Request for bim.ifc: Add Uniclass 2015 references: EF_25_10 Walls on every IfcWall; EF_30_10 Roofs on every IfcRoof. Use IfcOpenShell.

First a look at what the model holds.

```python
import ifcopenshell

model = ifcopenshell.open("bim.ifc")
print(model.schema)
print("classifications:", [c.Name for c in model.by_type("IfcClassification")])
for ifc_class in ("IfcDoor", "IfcRoof", "IfcStair", "IfcWall", "IfcWindow"):
    print(ifc_class, len(model.by_type(ifc_class)))
```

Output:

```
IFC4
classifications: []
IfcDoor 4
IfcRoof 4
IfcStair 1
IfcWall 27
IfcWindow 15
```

```python
import ifcopenshell
import ifcopenshell.api.classification

model = ifcopenshell.open("bim.ifc")

system = ifcopenshell.api.classification.add_classification(model, classification="Uniclass 2015")

codes = {
    "IfcWall": ("EF_25_10", "Walls"),
    "IfcRoof": ("EF_30_10", "Roofs"),
}
for ifc_class, (code, name) in codes.items():
    products = model.by_type(ifc_class)
    ifcopenshell.api.classification.add_reference(
        model, products=products, classification=system, identification=code, name=name
    )
    print(code, len(products))

model.write("bim_edited.ifc")
```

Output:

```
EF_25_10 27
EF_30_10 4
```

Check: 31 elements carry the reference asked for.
